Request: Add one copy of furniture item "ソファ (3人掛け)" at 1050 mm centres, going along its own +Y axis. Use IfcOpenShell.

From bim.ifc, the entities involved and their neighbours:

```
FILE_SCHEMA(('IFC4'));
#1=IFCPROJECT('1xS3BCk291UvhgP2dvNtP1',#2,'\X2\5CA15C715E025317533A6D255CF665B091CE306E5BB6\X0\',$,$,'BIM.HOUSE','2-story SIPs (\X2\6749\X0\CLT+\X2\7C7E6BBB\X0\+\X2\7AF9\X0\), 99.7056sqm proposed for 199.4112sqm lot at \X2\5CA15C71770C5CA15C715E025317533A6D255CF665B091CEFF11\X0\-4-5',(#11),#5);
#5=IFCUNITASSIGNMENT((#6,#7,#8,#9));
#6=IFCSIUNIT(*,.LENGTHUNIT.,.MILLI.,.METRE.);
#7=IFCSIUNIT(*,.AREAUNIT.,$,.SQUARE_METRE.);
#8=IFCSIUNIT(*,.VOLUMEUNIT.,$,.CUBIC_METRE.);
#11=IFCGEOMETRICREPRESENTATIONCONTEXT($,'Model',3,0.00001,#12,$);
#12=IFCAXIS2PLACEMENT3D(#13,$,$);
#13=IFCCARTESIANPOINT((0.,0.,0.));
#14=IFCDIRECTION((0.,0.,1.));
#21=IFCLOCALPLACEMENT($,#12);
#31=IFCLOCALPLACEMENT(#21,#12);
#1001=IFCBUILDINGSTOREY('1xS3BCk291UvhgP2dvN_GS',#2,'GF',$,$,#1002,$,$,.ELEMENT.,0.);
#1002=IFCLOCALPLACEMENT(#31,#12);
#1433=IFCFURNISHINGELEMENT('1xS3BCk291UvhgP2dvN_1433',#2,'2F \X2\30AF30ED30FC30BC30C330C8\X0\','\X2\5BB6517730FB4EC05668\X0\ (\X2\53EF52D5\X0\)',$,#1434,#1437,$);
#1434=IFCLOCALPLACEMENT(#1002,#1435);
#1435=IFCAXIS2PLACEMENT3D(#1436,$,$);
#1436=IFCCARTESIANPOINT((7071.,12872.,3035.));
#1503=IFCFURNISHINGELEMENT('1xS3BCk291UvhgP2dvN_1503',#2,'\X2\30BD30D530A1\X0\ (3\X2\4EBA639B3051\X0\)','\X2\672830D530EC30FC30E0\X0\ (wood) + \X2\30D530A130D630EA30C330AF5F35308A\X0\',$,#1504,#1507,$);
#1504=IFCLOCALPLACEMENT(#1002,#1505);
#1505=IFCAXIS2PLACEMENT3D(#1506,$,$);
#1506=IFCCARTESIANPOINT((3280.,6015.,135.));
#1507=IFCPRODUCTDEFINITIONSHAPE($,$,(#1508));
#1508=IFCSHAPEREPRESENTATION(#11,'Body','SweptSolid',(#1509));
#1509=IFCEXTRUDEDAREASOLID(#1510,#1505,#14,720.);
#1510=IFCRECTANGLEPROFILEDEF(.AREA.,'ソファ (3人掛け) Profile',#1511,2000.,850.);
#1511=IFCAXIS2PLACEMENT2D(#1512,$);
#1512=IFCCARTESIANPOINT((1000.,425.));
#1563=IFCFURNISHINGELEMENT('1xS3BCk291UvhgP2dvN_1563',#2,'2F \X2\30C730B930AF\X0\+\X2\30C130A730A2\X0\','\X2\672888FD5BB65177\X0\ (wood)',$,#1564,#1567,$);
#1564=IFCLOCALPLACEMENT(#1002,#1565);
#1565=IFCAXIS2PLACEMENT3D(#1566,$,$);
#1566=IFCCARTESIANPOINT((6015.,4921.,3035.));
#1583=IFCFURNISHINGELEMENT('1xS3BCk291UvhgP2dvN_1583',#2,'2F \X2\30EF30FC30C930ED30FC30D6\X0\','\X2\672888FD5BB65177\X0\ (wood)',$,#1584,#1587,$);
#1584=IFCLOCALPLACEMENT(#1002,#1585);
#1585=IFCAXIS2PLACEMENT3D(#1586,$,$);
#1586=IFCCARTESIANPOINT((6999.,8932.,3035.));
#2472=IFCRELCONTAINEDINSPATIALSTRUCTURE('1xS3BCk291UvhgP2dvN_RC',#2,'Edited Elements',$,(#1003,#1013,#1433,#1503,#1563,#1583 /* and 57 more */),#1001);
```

```python
import ifcopenshell
import ifcopenshell.api.geometry
import ifcopenshell.api.root
import ifcopenshell.util.element
import ifcopenshell.util.placement
import ifcopenshell.util.unit

model = ifcopenshell.open("bim.ifc")
unit_scale = ifcopenshell.util.unit.calculate_unit_scale(model)


def reuse_history(source, copy):
    """copy_class also copies each property set's owner history, people and application; keep the originals."""
    for rel in copy.IsDefinedBy:
        if rel.is_a("IfcRelDefinesByProperties") and (history := rel.RelatingPropertyDefinition.OwnerHistory):
            rel.RelatingPropertyDefinition.OwnerHistory = source.OwnerHistory
            ifcopenshell.util.element.remove_deep2(model, history)


source = model.by_guid("1xS3BCk291UvhgP2dvN_1503")
base = ifcopenshell.util.placement.get_local_placement(source.ObjectPlacement)
step = base[:3, 1] * 1.05 / unit_scale

for i in range(1, 2):
    copy = ifcopenshell.api.root.copy_class(model, product=source)
    copy.Representation = ifcopenshell.util.element.copy_deep(
        model, source.Representation, exclude=["IfcGeometricRepresentationContext", "IfcRepresentationMap"]
    )
    reuse_history(source, copy)
    matrix = base.copy()
    matrix[:3, 3] += i * step
    print("added at", matrix[:3, 3].round(3) + 0.0)
    ifcopenshell.api.geometry.edit_object_placement(model, product=copy, matrix=matrix, is_si=False)

model.write("bim_rev.ifc")
```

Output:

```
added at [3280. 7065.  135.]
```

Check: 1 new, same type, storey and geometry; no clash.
